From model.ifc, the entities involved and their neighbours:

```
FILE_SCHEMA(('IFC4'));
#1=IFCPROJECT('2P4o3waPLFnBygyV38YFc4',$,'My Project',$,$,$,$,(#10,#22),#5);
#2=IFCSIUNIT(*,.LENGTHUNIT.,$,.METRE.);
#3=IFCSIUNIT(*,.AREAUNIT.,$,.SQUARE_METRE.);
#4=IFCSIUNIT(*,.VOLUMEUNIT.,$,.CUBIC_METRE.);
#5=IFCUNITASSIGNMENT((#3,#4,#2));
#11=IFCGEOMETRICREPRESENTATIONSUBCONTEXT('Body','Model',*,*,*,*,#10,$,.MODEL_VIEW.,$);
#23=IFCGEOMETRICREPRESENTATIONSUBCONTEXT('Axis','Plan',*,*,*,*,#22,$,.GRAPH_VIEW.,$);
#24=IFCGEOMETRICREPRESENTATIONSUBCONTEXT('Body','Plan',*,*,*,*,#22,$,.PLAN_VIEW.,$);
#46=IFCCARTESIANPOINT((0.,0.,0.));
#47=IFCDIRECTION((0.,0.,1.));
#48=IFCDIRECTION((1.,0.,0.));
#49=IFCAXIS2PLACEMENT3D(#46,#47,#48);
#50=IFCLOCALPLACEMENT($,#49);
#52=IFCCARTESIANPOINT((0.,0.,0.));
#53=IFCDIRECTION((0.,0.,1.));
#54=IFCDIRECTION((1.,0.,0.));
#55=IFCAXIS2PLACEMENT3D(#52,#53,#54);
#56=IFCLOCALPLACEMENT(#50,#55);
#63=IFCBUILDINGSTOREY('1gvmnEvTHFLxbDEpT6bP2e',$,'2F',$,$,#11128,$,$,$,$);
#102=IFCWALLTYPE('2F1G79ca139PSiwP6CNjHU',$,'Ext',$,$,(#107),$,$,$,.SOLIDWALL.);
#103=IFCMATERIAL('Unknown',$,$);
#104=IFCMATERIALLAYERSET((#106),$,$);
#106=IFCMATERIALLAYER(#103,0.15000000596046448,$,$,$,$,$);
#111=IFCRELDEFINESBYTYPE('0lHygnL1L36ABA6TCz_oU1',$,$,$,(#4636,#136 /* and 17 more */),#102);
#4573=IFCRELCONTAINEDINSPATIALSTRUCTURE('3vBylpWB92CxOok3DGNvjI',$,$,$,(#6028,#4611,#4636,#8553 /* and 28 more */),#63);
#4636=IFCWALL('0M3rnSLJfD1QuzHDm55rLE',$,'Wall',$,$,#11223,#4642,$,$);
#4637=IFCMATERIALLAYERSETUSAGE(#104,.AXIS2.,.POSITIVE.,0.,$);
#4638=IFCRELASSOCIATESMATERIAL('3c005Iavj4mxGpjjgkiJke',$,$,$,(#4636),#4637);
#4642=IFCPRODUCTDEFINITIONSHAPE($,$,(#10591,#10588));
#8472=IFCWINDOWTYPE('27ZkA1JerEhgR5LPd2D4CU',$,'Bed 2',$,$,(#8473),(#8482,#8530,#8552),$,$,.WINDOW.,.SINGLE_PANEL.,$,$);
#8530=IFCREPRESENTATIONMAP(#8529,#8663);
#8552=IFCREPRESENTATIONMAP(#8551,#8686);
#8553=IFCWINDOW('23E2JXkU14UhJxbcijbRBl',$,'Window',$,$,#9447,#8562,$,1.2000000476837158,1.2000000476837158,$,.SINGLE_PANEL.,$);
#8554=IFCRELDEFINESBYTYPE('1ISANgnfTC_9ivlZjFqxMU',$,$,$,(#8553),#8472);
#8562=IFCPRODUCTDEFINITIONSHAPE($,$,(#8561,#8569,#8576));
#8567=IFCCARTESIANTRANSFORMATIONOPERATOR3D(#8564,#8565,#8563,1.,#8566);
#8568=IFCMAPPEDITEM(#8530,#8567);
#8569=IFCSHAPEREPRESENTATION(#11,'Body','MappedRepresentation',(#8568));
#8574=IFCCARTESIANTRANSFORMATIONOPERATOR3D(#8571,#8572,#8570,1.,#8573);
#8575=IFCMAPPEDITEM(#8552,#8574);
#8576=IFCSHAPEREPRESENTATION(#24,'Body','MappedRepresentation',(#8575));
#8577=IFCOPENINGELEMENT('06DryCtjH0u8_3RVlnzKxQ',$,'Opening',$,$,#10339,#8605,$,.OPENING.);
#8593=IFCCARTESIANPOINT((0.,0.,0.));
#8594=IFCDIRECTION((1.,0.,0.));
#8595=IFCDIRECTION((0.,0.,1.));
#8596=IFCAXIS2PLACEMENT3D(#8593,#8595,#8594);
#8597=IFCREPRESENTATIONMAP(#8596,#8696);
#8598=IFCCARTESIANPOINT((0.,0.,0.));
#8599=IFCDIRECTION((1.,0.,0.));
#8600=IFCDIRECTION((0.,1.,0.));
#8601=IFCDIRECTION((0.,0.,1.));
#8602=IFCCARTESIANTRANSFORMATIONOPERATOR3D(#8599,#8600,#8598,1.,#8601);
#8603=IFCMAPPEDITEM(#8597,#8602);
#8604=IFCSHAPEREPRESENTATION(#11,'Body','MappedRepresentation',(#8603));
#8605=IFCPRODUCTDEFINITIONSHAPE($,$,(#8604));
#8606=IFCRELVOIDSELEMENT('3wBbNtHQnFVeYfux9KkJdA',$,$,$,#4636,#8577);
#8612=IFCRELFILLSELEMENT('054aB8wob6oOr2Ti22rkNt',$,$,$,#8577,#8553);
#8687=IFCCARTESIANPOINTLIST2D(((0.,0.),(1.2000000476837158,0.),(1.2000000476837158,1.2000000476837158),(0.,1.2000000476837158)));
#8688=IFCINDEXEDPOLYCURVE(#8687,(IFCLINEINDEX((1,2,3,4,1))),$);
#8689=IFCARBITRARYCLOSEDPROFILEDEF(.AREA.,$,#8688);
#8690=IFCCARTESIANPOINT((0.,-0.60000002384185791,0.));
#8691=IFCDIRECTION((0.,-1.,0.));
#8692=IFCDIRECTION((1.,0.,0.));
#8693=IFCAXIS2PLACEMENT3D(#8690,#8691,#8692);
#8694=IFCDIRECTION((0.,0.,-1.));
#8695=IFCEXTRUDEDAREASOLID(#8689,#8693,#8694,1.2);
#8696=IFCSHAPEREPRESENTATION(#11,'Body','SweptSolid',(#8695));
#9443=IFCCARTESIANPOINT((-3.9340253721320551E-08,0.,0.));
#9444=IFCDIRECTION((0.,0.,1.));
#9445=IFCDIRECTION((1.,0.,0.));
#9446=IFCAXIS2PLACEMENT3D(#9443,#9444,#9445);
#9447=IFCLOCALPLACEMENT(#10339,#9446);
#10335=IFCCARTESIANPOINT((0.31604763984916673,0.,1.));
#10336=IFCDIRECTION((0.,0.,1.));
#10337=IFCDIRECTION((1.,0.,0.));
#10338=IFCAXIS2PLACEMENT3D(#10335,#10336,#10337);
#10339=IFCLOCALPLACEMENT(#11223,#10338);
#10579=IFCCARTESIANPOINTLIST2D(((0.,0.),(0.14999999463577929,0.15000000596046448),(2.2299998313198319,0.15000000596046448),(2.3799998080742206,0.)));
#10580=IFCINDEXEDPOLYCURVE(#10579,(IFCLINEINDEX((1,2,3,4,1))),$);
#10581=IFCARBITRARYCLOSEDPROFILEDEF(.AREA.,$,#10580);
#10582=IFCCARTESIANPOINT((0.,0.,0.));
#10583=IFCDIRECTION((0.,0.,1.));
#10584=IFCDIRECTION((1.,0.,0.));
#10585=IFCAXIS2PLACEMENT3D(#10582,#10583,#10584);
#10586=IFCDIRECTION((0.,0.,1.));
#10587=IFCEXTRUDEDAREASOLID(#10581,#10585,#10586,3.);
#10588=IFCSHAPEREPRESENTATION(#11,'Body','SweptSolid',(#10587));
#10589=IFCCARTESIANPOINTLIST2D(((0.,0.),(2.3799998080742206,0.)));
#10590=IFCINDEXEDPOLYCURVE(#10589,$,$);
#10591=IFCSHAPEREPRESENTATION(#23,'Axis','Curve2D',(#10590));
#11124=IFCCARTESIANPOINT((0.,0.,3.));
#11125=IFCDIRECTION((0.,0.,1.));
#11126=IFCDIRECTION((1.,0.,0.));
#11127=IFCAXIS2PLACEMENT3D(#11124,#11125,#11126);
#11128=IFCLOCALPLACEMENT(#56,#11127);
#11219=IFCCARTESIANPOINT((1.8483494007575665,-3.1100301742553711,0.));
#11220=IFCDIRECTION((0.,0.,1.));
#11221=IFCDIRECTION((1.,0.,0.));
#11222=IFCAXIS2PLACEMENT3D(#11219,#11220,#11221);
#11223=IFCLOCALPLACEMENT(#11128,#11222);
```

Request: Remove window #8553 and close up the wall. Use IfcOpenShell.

```python
import ifcopenshell
import ifcopenshell.api.feature
import ifcopenshell.api.root
import ifcopenshell.geom
import ifcopenshell.util.shape

model = ifcopenshell.open("model.ifc")
settings = ifcopenshell.geom.settings()


def volume(element):
    """Net volume in cubic metres, openings subtracted."""
    shape = ifcopenshell.geom.create_shape(settings, element)
    return ifcopenshell.util.shape.get_volume(shape.geometry)


window = model.by_guid("23E2JXkU14UhJxbcijbRBl")
opening = window.FillsVoids[0].RelatingOpeningElement
wall = opening.VoidsElements[0].RelatingBuildingElement
before = volume(wall)

ifcopenshell.api.root.remove_product(model, product=window)
ifcopenshell.api.feature.remove_feature(model, feature=opening)

after = volume(wall)

print(f"wall volume {before:.3f} -> {after:.3f} m3")

model.write("model_edited.ifc")
```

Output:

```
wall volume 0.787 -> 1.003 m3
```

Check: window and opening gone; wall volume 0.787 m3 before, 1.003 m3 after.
